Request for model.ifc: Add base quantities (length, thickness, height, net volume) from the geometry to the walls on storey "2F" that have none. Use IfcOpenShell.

First a look at what the model holds.

```python
import ifcopenshell
import ifcopenshell.util.element
import ifcopenshell.util.unit

model = ifcopenshell.open("model.ifc")
print(model.schema)
for unit_type in ("LENGTHUNIT", "AREAUNIT", "VOLUMEUNIT"):
    print(unit_type, ifcopenshell.util.unit.calculate_unit_scale(model, unit_type))
storey = next(s for s in model.by_type("IfcBuildingStorey") if s.Name == "2F")
walls = [e for e in ifcopenshell.util.element.get_decomposition(storey) if e.is_a("IfcWall")]
for e in sorted(walls, key=lambda e: e.id()):
    print(e.id(), e.is_a(), e.Name, list(ifcopenshell.util.element.get_psets(e, qtos_only=True)), sep=" | ")
```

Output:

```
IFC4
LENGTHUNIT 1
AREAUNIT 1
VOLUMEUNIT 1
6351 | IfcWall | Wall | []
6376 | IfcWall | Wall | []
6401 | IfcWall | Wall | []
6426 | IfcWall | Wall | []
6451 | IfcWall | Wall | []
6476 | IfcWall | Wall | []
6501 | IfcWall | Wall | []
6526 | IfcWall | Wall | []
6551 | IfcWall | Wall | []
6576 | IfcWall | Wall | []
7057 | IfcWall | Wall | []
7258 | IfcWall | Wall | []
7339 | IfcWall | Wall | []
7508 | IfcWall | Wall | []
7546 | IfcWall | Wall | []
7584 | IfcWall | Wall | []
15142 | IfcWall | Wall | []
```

```python
import ifcopenshell
import ifcopenshell.api.pset
import ifcopenshell.geom
import ifcopenshell.util.element
import ifcopenshell.util.shape
import ifcopenshell.util.unit

model = ifcopenshell.open("model.ifc")
unit_scale = ifcopenshell.util.unit.calculate_unit_scale(model)
volume_scale = ifcopenshell.util.unit.calculate_unit_scale(model, "VOLUMEUNIT")
settings = ifcopenshell.geom.settings()

storey = next(s for s in model.by_type("IfcBuildingStorey") if s.Name == "2F")
walls = [e for e in ifcopenshell.util.element.get_decomposition(storey) if e.is_a("IfcWall")]

for e in sorted(walls, key=lambda e: e.id()):
    if ifcopenshell.util.element.get_psets(e, qtos_only=True, should_inherit=False):
        continue
    # Geometry comes back in metres, in the element's own axes.
    shape = ifcopenshell.geom.create_shape(settings, e)
    values = {
        "Length": ifcopenshell.util.shape.get_x(shape.geometry) / unit_scale,
        "Width": ifcopenshell.util.shape.get_y(shape.geometry) / unit_scale,
        "Height": ifcopenshell.util.shape.get_z(shape.geometry) / unit_scale,
        "NetVolume": ifcopenshell.util.shape.get_volume(shape.geometry) / volume_scale,
    }
    qto = ifcopenshell.api.pset.add_qto(model, product=e, name="Qto_WallBaseQuantities")
    ifcopenshell.api.pset.edit_qto(model, qto=qto, properties=values)
    print(e.id(), {k: round(v, 3) for k, v in values.items()})

model.write("model_updated.ifc")
```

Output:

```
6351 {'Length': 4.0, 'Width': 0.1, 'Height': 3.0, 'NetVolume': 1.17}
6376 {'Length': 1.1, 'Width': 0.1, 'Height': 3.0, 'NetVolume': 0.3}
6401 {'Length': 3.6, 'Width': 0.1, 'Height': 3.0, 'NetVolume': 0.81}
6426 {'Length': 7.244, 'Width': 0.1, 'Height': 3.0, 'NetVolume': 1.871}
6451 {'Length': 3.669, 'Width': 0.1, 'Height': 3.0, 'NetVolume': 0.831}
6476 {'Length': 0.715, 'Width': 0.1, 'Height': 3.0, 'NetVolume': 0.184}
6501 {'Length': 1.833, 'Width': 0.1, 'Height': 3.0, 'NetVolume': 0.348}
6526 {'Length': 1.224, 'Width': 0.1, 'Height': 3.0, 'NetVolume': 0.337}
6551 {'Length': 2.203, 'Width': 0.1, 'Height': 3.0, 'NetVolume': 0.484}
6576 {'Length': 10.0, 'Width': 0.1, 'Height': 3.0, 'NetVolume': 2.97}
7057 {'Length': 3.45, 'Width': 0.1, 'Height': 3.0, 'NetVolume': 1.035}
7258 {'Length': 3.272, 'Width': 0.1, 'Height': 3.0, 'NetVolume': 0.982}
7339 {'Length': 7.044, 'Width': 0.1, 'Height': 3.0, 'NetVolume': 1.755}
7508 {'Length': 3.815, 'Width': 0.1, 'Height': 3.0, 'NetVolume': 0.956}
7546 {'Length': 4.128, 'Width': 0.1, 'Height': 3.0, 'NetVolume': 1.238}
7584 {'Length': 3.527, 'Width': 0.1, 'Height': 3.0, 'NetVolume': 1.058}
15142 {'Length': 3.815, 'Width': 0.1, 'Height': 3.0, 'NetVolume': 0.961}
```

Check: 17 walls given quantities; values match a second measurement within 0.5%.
